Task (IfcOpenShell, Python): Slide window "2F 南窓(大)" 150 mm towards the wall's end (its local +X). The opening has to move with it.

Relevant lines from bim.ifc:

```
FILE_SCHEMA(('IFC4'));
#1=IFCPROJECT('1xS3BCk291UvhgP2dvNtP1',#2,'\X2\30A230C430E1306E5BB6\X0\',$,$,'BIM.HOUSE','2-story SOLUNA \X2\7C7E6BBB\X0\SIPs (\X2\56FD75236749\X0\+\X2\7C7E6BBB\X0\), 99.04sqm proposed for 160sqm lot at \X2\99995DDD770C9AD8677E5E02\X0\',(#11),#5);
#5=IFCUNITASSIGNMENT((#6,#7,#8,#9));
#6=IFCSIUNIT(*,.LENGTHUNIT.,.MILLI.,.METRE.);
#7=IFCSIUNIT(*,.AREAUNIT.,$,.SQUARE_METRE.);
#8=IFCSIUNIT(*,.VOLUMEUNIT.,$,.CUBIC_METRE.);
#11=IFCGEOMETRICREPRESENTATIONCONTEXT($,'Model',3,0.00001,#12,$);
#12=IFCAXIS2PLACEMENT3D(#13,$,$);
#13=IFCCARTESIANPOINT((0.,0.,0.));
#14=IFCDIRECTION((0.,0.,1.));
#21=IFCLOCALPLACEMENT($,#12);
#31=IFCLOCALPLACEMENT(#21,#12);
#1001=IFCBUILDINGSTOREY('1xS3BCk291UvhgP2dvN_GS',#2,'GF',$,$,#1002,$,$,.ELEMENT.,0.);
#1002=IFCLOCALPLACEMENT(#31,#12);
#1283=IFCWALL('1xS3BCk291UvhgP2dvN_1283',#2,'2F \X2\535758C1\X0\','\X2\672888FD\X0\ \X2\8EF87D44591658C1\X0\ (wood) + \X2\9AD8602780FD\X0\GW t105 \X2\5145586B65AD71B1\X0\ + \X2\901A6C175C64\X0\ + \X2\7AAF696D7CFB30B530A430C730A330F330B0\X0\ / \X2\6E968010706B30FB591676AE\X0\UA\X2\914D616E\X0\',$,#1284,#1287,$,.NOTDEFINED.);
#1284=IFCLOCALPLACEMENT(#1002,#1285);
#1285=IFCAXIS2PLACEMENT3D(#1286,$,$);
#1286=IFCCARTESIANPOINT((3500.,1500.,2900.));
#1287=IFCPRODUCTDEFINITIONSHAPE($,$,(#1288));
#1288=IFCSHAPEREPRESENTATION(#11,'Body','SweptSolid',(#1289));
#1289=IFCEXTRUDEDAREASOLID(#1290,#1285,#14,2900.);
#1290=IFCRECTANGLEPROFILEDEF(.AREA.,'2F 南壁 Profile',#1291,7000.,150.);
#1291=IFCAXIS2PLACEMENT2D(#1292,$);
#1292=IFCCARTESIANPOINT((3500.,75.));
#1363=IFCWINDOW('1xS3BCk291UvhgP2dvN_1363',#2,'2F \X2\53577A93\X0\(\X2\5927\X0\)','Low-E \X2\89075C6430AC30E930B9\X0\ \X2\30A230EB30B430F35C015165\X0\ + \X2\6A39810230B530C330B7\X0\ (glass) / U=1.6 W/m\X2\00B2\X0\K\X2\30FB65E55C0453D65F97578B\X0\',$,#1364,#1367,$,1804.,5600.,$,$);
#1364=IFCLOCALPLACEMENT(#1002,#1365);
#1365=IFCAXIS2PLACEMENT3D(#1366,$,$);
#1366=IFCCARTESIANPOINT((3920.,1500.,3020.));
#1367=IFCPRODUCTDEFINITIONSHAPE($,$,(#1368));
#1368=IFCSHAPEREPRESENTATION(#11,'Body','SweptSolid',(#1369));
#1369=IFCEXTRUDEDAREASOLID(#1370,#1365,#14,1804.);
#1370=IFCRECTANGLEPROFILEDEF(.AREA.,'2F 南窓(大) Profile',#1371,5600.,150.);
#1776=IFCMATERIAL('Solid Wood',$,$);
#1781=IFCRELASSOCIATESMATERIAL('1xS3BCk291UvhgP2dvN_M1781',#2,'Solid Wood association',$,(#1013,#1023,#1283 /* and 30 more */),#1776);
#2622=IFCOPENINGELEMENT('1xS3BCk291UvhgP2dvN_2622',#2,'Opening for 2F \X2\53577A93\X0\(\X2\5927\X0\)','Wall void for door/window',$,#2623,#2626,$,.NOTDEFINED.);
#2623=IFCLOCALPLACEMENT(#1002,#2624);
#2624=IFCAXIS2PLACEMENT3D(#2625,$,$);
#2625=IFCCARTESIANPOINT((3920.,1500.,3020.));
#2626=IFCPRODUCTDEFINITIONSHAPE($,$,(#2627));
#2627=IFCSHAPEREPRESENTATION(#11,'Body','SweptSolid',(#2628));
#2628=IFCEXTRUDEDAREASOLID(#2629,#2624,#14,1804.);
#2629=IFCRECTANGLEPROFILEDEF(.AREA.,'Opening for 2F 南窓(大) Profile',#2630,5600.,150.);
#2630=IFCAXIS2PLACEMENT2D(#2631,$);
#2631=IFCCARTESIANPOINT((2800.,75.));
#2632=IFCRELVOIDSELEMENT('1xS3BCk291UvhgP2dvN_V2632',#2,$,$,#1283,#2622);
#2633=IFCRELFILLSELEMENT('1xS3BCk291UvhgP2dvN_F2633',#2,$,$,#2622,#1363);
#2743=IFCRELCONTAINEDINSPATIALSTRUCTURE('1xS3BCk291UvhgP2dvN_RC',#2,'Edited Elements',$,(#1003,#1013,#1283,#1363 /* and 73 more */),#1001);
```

```python
import ifcopenshell
import ifcopenshell.api.geometry
import ifcopenshell.util.placement

model = ifcopenshell.open("bim.ifc")

window = model.by_guid("1xS3BCk291UvhgP2dvN_1363")
opening = window.FillsVoids[0].RelatingOpeningElement
wall = opening.VoidsElements[0].RelatingBuildingElement

wall_matrix = ifcopenshell.util.placement.get_local_placement(wall.ObjectPlacement)
shift = wall_matrix[:3, 0] * 150.0
before = ifcopenshell.util.placement.get_local_placement(window.ObjectPlacement)[:3, 3].copy()

# The window is not placed relative to its opening, so move both.
for product in (opening, window):
    matrix = ifcopenshell.util.placement.get_local_placement(product.ObjectPlacement)
    matrix[:3, 3] += shift
    ifcopenshell.api.geometry.edit_object_placement(model, product=product, matrix=matrix, is_si=False)

after = ifcopenshell.util.placement.get_local_placement(window.ObjectPlacement)[:3, 3]
print("window moved by", (after - before).round(3) + 0.0)

model.write("bim_updated.ifc")
```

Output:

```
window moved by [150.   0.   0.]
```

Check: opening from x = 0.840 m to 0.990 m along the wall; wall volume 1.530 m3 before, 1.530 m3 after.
